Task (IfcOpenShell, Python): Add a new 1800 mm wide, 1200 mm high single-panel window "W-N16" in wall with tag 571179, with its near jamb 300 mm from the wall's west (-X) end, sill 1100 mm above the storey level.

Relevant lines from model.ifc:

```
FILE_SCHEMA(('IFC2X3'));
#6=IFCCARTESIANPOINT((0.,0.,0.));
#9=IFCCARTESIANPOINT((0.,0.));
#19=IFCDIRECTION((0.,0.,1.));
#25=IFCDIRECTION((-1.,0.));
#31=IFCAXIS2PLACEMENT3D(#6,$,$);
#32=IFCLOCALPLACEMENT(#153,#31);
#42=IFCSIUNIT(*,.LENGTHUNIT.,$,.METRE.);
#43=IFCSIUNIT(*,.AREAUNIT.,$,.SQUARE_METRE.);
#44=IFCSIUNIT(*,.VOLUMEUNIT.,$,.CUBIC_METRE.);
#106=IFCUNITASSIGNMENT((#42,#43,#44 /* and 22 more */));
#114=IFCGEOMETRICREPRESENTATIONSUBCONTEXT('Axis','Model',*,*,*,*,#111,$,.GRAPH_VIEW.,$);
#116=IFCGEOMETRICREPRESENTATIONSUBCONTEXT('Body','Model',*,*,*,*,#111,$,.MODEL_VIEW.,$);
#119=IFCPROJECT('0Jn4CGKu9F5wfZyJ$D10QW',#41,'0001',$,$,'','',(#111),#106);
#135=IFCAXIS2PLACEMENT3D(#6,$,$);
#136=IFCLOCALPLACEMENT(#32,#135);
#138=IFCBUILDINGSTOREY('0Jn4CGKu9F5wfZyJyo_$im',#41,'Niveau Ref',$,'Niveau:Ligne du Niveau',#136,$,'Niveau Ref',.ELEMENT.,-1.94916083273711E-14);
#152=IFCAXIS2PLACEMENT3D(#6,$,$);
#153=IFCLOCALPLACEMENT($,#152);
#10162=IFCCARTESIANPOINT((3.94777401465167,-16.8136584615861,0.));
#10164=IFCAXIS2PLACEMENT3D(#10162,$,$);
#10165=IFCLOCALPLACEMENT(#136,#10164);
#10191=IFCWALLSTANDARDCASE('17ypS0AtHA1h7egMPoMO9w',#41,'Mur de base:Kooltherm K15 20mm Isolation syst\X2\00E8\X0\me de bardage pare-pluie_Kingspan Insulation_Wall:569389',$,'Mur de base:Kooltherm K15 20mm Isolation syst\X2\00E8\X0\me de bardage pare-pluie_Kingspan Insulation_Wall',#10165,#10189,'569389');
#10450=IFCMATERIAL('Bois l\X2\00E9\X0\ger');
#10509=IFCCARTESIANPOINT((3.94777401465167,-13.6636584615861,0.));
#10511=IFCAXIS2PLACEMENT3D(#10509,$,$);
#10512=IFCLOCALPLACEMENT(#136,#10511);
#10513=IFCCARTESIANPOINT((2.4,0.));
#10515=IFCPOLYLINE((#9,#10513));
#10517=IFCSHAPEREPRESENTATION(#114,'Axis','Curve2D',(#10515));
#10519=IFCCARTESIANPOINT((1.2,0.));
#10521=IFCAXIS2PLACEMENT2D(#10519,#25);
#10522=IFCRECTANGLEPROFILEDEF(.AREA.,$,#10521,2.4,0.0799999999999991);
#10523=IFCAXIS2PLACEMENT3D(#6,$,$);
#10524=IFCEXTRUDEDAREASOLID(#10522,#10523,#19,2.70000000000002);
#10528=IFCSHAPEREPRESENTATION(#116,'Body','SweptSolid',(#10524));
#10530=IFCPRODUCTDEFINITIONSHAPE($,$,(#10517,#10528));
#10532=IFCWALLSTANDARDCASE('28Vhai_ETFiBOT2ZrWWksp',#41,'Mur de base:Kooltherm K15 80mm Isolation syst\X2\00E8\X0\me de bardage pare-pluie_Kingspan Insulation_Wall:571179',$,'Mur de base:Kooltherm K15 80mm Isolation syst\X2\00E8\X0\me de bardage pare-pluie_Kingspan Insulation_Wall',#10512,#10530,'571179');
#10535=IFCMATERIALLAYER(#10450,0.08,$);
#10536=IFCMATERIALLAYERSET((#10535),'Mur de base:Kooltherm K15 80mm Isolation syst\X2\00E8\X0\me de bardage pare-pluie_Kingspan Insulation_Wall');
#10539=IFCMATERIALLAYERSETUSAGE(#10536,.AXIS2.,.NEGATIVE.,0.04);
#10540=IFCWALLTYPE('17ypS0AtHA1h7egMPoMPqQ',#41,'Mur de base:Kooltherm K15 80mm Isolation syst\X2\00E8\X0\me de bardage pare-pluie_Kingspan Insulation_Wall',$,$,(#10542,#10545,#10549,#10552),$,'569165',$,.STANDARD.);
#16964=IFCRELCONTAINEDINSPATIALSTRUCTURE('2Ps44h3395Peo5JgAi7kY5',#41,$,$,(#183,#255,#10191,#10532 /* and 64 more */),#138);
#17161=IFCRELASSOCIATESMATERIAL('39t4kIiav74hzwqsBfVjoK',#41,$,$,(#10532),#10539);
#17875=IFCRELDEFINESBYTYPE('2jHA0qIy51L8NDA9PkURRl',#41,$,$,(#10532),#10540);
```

```python
import numpy as np
import ifcopenshell
import ifcopenshell.api.feature
import ifcopenshell.api.geometry
import ifcopenshell.api.root
import ifcopenshell.api.spatial
import ifcopenshell.api.type
import ifcopenshell.geom
import ifcopenshell.util.element
import ifcopenshell.util.placement
import ifcopenshell.util.representation
import ifcopenshell.util.shape
import ifcopenshell.util.unit

model = ifcopenshell.open("model.ifc")
unit_scale = ifcopenshell.util.unit.calculate_unit_scale(model)
settings = ifcopenshell.geom.settings()


def volume(element):
    """Net volume in cubic metres, openings subtracted."""
    shape = ifcopenshell.geom.create_shape(settings, element)
    return ifcopenshell.util.shape.get_volume(shape.geometry)


wall = model.by_guid("28Vhai_ETFiBOT2ZrWWksp")
storey = ifcopenshell.util.element.get_container(wall, ifc_class="IfcBuildingStorey")
context = ifcopenshell.util.representation.get_context(model, "Model", "Body", "MODEL_VIEW")
before = volume(wall)

width, height, from_end, sill = 1.8, 1.2, 0.3, 1.1  # metres

# The wall runs along its own X axis, and the end named is its -X end.
wall_shape = ifcopenshell.geom.create_shape(settings, wall)
x, y, z = ifcopenshell.util.shape.get_vertices(wall_shape.geometry).T
start = x.min() + from_end
face, thickness = float(y.min()), float(y.max() - y.min())
wall_matrix = ifcopenshell.util.placement.get_local_placement(wall.ObjectPlacement)
level = ifcopenshell.util.placement.get_local_placement(storey.ObjectPlacement)[2, 3]


def in_wall(x, y):
    """Placement at x, y metres in the wall's axes, at sill height."""
    matrix = wall_matrix.copy()
    matrix[:, 3] = wall_matrix @ np.array([x / unit_scale, y / unit_scale, 0.0, 1.0])
    matrix[2, 3] = level + sill / unit_scale
    return matrix


# Opening: a box that overshoots both wall faces by 50 mm.
opening = ifcopenshell.api.root.create_entity(model, ifc_class="IfcOpeningElement")
box = ifcopenshell.api.geometry.add_wall_representation(
    model, context=context, length=width, height=height, thickness=thickness + 0.1
)
ifcopenshell.api.geometry.assign_representation(model, product=opening, representation=box)
ifcopenshell.api.geometry.edit_object_placement(model, product=opening, matrix=in_wall(start, face - 0.05), is_si=False)
ifcopenshell.api.feature.add_feature(model, feature=opening, element=wall)

window = ifcopenshell.api.root.create_entity(model, ifc_class="IfcWindow", name="W-N16")
window.OverallWidth, window.OverallHeight = width / unit_scale, height / unit_scale
body = ifcopenshell.api.geometry.add_window_representation(
    model,
    context=context,
    overall_width=window.OverallWidth,
    overall_height=window.OverallHeight,
    partition_type="SINGLE_PANEL",
)
ifcopenshell.api.geometry.assign_representation(model, product=window, representation=body)
ifcopenshell.api.spatial.assign_container(model, products=[window], relating_structure=storey)
fills = ifcopenshell.api.feature.add_filling(model, opening=opening, element=window)
fills.OwnerHistory = window.OwnerHistory  # required in IFC2X3

# IFC2X3 keeps the operation on the window style.
style = ifcopenshell.api.root.create_entity(model, ifc_class="IfcWindowStyle", name="W-N16")
style.OperationType, style.ConstructionType = "SINGLE_PANEL", "NOTDEFINED"
style.ParameterTakesPrecedence = style.Sizeable = False
ifcopenshell.api.type.assign_type(model, related_objects=[window], relating_type=style)

# Centre the window in the wall's thickness.
ifcopenshell.api.geometry.edit_object_placement(model, product=window, matrix=in_wall(start, face), is_si=False)
window_shape = ifcopenshell.geom.create_shape(settings, window)
depth = ifcopenshell.util.shape.get_vertices(window_shape.geometry)[:, 1]
offset = face + thickness / 2 - (depth.min() + depth.max()) / 2
ifcopenshell.api.geometry.edit_object_placement(model, product=window, matrix=in_wall(start, offset), is_si=False)

after = volume(wall)

print(f"wall volume {before:.3f} -> {after:.3f} m3")

model.write("model_updated.ifc")
```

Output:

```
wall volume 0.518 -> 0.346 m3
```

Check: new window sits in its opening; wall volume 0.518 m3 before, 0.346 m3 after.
